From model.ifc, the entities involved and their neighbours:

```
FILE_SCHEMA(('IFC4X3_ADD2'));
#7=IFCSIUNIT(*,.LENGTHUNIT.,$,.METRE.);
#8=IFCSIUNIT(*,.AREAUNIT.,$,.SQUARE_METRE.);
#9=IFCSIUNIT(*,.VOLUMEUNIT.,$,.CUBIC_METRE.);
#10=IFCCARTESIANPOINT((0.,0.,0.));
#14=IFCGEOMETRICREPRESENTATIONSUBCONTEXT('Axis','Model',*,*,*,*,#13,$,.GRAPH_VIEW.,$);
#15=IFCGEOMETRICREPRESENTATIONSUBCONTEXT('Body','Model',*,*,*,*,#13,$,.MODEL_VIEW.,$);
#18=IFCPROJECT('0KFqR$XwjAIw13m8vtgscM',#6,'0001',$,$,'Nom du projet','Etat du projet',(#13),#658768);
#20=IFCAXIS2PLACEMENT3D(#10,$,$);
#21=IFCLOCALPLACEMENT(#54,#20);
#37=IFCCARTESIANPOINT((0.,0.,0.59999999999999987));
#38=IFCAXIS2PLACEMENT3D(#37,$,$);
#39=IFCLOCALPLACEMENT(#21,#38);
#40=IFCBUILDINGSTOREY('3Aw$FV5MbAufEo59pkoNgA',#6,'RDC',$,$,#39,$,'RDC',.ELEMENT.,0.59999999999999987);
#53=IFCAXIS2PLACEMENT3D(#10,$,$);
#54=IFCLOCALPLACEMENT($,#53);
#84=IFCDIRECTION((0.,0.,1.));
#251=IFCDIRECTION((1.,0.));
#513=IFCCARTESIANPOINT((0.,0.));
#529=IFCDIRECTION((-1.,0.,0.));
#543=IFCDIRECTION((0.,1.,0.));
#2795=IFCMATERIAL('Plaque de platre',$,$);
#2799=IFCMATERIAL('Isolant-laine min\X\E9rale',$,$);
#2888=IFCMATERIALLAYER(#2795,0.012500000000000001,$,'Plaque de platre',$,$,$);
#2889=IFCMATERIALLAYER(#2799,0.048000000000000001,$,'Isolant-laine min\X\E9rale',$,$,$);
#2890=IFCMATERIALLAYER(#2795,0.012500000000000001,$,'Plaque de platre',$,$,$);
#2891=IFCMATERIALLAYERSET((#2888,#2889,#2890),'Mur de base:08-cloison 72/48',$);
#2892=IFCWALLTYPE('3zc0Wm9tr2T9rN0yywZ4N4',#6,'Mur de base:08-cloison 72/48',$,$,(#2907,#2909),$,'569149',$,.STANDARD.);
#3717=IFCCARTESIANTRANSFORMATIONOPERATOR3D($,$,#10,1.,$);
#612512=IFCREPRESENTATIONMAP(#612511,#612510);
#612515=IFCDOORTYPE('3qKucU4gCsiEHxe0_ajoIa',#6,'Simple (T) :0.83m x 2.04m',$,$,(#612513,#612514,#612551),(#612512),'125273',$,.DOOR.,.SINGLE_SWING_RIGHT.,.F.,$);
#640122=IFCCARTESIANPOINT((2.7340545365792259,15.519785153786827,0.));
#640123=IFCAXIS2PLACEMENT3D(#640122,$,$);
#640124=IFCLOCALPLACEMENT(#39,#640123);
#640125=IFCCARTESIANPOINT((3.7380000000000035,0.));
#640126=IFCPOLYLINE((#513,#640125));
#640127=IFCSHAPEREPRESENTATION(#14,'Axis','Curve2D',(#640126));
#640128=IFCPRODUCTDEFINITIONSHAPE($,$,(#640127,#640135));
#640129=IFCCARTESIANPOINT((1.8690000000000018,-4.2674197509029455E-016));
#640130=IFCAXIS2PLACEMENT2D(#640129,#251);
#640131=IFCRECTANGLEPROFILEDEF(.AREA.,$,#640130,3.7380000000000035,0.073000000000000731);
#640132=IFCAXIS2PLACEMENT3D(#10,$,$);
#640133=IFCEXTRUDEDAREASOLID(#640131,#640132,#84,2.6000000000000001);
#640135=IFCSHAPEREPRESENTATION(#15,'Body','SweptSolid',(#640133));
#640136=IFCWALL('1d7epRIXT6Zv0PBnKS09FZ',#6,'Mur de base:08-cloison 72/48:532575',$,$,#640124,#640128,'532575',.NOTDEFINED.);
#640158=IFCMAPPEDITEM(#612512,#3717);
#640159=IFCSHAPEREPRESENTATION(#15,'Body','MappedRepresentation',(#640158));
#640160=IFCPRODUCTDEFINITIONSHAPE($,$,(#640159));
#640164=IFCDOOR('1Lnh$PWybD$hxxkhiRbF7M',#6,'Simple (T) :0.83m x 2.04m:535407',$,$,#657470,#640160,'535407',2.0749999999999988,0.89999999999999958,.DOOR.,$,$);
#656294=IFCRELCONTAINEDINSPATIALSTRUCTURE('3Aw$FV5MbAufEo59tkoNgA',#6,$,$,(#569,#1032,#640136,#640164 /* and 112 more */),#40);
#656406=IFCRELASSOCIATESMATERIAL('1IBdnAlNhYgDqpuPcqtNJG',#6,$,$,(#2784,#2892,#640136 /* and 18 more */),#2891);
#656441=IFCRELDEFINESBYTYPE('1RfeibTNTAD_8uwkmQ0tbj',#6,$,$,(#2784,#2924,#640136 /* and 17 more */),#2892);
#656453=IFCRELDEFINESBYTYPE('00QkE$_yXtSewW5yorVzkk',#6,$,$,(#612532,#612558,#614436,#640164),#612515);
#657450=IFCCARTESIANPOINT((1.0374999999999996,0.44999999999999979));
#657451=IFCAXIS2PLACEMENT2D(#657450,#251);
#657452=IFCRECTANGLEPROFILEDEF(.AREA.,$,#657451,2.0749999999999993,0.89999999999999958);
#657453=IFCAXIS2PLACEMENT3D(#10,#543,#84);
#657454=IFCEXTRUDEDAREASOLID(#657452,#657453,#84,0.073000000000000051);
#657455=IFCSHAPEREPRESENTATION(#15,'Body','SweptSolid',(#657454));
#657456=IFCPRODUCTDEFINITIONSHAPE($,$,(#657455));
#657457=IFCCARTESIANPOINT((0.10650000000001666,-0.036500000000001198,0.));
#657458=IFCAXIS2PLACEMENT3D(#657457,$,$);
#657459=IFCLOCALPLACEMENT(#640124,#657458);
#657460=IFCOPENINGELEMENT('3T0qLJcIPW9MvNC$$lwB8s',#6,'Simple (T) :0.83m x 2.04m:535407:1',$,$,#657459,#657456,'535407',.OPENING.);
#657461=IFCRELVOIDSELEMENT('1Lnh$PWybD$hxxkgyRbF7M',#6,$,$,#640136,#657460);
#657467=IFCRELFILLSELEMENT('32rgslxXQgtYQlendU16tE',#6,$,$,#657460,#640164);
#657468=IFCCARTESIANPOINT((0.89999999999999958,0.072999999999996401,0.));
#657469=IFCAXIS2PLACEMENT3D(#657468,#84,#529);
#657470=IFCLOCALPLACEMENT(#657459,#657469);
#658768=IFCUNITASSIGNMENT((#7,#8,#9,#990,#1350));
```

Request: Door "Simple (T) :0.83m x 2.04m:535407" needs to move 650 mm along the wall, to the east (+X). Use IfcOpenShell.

```python
import ifcopenshell
import ifcopenshell.api.geometry
import ifcopenshell.util.placement
import ifcopenshell.util.unit

model = ifcopenshell.open("model.ifc")
unit_scale = ifcopenshell.util.unit.calculate_unit_scale(model)

door = model.by_guid("1Lnh$PWybD$hxxkhiRbF7M")
opening = door.FillsVoids[0].RelatingOpeningElement
wall = opening.VoidsElements[0].RelatingBuildingElement

wall_matrix = ifcopenshell.util.placement.get_local_placement(wall.ObjectPlacement)
shift = wall_matrix[:3, 0] * 0.65 / unit_scale
before = ifcopenshell.util.placement.get_local_placement(door.ObjectPlacement)[:3, 3].copy()

# The door is placed relative to its opening, so it follows when the opening moves.
matrix = ifcopenshell.util.placement.get_local_placement(opening.ObjectPlacement)
matrix[:3, 3] += shift
ifcopenshell.api.geometry.edit_object_placement(
    model, product=opening, matrix=matrix, is_si=False, should_transform_children=True
)

after = ifcopenshell.util.placement.get_local_placement(door.ObjectPlacement)[:3, 3]
print("door moved by", (after - before).round(3) + 0.0)

model.write("model_updated.ifc")
```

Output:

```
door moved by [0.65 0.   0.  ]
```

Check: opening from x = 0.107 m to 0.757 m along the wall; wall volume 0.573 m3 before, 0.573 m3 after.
